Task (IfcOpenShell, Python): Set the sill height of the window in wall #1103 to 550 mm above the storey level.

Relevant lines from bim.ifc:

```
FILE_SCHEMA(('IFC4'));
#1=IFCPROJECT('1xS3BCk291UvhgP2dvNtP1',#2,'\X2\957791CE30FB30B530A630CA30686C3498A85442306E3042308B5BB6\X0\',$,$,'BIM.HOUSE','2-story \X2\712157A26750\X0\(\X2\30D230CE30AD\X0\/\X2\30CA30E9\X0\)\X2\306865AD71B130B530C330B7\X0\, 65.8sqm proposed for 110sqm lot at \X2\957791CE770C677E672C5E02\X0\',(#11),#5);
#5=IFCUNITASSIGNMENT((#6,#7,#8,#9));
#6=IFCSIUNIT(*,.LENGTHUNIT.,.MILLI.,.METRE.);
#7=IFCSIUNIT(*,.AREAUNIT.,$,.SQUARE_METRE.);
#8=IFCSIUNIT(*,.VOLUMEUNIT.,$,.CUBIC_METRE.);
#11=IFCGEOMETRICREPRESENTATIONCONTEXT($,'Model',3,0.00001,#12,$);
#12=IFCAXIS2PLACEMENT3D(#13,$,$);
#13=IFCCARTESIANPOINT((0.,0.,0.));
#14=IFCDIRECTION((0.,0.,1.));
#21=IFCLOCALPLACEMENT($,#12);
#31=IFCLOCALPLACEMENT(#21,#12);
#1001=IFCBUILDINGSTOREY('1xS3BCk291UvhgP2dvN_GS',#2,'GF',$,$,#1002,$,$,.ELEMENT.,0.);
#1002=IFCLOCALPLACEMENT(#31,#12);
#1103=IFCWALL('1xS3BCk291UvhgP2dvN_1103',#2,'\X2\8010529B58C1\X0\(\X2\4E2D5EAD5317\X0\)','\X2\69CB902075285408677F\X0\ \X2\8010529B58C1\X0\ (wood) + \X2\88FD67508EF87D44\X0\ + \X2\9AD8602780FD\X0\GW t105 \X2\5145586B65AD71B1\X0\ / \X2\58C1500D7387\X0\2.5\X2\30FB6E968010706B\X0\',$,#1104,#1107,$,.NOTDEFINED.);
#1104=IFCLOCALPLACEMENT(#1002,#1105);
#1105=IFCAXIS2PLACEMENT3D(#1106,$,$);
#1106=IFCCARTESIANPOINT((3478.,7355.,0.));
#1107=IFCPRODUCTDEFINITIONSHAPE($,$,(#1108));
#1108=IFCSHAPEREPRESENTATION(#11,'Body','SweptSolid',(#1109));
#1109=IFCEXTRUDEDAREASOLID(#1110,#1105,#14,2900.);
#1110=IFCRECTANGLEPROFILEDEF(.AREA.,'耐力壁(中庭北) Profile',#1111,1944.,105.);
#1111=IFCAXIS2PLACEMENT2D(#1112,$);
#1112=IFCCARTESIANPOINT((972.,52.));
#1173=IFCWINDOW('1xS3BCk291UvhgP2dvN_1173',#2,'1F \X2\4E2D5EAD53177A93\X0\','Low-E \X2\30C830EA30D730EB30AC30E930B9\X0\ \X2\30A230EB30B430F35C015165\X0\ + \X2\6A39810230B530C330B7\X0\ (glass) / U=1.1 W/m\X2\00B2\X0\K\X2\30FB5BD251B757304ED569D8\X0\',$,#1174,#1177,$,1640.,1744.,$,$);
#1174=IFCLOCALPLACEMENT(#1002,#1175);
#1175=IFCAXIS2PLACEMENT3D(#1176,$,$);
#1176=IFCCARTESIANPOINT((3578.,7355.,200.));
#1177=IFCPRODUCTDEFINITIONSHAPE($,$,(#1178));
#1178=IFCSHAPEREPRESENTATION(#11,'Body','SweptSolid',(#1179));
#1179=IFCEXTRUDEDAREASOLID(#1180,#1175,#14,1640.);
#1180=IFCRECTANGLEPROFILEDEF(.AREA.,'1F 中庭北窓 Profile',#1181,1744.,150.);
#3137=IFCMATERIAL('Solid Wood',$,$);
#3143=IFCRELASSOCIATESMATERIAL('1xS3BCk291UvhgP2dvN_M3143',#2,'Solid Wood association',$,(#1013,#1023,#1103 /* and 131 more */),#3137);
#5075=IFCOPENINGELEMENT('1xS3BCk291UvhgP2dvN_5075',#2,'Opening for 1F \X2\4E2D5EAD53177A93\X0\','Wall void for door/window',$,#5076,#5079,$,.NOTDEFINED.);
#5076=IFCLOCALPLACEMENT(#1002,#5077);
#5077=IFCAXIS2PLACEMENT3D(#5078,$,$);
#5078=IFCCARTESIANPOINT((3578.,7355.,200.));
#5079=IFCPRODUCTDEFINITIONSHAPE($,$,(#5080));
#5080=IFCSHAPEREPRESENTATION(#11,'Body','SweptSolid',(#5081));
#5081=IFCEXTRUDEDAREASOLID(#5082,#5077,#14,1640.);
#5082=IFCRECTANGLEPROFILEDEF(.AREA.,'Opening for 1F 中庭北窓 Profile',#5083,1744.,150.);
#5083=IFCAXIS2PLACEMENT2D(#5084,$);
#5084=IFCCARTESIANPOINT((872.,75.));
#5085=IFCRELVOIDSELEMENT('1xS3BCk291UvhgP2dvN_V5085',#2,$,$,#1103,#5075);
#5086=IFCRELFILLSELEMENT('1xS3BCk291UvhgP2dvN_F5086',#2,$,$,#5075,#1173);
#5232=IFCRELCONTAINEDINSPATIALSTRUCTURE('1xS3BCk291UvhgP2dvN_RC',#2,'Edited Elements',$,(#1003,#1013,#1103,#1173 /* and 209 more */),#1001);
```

```python
import numpy as np
import ifcopenshell
import ifcopenshell.api.geometry
import ifcopenshell.geom
import ifcopenshell.util.element
import ifcopenshell.util.placement
import ifcopenshell.util.shape
import ifcopenshell.util.unit

model = ifcopenshell.open("bim.ifc")
unit_scale = ifcopenshell.util.unit.calculate_unit_scale(model)

window = model.by_id(1173)
opening = window.FillsVoids[0].RelatingOpeningElement
storey = ifcopenshell.util.element.get_container(window, ifc_class="IfcBuildingStorey")
level = ifcopenshell.util.placement.get_local_placement(storey.ObjectPlacement)[2, 3]

# The opening's origin need not be at the sill, so measure its lowest point.
shape = ifcopenshell.geom.create_shape(ifcopenshell.geom.settings(), opening)
bottom = ifcopenshell.util.shape.get_shape_bottom_elevation(shape, shape.geometry) / unit_scale
dz = level + 550.0 - bottom

shift = np.array([0.0, 0.0, dz])
# The window is not placed relative to its opening, so move both.
for product in (opening, window):
    matrix = ifcopenshell.util.placement.get_local_placement(product.ObjectPlacement)
    matrix[:3, 3] += shift
    ifcopenshell.api.geometry.edit_object_placement(model, product=product, matrix=matrix, is_si=False)

print(f"moved by {dz * unit_scale:+.3f} m")

model.write("bim-out.ifc")
```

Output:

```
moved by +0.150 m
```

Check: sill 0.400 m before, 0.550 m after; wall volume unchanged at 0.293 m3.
